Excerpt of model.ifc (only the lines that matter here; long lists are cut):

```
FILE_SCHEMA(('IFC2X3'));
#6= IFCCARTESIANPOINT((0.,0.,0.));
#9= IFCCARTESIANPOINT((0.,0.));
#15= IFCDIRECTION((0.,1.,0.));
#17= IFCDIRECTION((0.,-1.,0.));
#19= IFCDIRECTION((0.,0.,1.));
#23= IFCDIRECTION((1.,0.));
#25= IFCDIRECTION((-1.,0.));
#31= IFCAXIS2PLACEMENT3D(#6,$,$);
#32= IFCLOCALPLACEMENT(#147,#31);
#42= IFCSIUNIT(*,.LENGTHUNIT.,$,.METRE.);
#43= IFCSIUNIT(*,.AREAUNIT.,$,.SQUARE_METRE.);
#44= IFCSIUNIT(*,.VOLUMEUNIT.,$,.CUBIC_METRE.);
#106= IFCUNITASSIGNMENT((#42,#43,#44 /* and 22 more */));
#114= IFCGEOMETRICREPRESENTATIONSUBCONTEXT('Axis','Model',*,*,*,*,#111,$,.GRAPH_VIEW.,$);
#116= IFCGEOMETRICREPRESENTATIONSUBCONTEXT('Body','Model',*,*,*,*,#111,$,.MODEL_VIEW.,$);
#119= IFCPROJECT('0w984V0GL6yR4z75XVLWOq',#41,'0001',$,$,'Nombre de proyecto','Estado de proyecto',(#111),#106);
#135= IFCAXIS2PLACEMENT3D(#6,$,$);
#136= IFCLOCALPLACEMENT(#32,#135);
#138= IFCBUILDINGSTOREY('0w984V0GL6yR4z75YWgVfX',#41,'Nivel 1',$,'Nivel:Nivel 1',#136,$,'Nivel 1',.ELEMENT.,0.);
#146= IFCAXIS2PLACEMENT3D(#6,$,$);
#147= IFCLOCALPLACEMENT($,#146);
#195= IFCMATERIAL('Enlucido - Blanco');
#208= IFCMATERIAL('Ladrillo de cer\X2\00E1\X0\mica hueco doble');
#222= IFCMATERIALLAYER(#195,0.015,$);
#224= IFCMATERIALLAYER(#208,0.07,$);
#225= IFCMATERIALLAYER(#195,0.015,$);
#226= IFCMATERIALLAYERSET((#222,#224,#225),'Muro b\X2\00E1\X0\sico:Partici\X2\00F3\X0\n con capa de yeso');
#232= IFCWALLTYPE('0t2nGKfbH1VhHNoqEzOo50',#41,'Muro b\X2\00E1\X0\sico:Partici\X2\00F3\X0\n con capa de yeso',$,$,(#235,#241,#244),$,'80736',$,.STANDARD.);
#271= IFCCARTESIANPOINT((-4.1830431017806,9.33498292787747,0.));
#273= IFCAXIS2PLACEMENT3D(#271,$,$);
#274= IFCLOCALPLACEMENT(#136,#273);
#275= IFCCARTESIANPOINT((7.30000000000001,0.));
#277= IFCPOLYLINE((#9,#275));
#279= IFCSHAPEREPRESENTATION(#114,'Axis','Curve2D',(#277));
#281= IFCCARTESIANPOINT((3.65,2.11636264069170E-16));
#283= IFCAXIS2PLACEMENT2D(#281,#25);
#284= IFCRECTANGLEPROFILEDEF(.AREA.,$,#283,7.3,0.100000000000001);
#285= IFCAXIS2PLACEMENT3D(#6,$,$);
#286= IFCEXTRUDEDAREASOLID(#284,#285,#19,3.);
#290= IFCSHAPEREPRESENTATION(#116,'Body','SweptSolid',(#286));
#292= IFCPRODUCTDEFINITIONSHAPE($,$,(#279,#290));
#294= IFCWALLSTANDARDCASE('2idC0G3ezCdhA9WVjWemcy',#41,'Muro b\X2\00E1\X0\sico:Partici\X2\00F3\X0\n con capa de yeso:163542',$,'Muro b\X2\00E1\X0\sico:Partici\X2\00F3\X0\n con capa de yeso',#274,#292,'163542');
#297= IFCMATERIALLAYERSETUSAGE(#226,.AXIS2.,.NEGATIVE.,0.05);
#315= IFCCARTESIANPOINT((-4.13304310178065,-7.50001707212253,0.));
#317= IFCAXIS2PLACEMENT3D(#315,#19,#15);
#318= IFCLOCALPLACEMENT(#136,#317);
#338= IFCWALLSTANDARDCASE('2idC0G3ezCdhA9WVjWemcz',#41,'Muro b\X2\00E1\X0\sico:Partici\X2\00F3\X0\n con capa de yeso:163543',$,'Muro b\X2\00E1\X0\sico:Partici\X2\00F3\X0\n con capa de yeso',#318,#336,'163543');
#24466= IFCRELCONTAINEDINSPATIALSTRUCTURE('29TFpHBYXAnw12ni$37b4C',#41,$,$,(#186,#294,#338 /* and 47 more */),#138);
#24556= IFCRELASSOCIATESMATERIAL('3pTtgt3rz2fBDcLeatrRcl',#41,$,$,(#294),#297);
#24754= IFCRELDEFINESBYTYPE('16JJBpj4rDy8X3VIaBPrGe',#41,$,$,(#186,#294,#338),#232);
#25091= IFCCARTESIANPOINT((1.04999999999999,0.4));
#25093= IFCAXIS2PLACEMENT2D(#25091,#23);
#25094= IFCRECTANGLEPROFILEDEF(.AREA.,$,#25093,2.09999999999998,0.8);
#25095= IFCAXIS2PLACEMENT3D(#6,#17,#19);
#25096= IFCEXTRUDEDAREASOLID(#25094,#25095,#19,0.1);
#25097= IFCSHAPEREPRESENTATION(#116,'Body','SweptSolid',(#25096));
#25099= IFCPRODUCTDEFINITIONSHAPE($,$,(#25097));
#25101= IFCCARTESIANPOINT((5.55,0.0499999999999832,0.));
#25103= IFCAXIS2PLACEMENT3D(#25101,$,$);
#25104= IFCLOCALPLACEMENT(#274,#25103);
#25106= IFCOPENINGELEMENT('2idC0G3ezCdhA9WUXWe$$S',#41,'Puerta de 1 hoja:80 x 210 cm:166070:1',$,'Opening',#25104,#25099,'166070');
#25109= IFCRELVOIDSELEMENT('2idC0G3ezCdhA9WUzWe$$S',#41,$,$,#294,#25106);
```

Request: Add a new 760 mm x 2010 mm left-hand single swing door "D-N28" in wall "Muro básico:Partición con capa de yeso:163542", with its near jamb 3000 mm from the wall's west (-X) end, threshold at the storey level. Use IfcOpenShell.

```python
import numpy as np
import ifcopenshell
import ifcopenshell.api.feature
import ifcopenshell.api.geometry
import ifcopenshell.api.root
import ifcopenshell.api.spatial
import ifcopenshell.api.type
import ifcopenshell.geom
import ifcopenshell.util.element
import ifcopenshell.util.placement
import ifcopenshell.util.representation
import ifcopenshell.util.shape
import ifcopenshell.util.unit

model = ifcopenshell.open("model.ifc")
unit_scale = ifcopenshell.util.unit.calculate_unit_scale(model)
settings = ifcopenshell.geom.settings()


def volume(element):
    """Net volume in cubic metres, openings subtracted."""
    shape = ifcopenshell.geom.create_shape(settings, element)
    return ifcopenshell.util.shape.get_volume(shape.geometry)


wall = model.by_guid("2idC0G3ezCdhA9WVjWemcy")
storey = ifcopenshell.util.element.get_container(wall, ifc_class="IfcBuildingStorey")
context = ifcopenshell.util.representation.get_context(model, "Model", "Body", "MODEL_VIEW")
before = volume(wall)

width, height, from_end, sill = 0.76, 2.01, 3, 0.0  # metres

# The wall runs along its own X axis, and the end named is its -X end.
wall_shape = ifcopenshell.geom.create_shape(settings, wall)
x, y, z = ifcopenshell.util.shape.get_vertices(wall_shape.geometry).T
start = x.min() + from_end
face, thickness = float(y.min()), float(y.max() - y.min())
wall_matrix = ifcopenshell.util.placement.get_local_placement(wall.ObjectPlacement)
level = ifcopenshell.util.placement.get_local_placement(storey.ObjectPlacement)[2, 3]


def in_wall(x, y):
    """Placement at x, y metres in the wall's axes, at sill height."""
    matrix = wall_matrix.copy()
    matrix[:, 3] = wall_matrix @ np.array([x / unit_scale, y / unit_scale, 0.0, 1.0])
    matrix[2, 3] = level + sill / unit_scale
    return matrix


# Opening: a box that overshoots both wall faces by 50 mm.
opening = ifcopenshell.api.root.create_entity(model, ifc_class="IfcOpeningElement")
box = ifcopenshell.api.geometry.add_wall_representation(
    model, context=context, length=width, height=height, thickness=thickness + 0.1
)
ifcopenshell.api.geometry.assign_representation(model, product=opening, representation=box)
ifcopenshell.api.geometry.edit_object_placement(model, product=opening, matrix=in_wall(start, face - 0.05), is_si=False)
ifcopenshell.api.feature.add_feature(model, feature=opening, element=wall)

door = ifcopenshell.api.root.create_entity(model, ifc_class="IfcDoor", name="D-N28")
door.OverallWidth, door.OverallHeight = width / unit_scale, height / unit_scale
body = ifcopenshell.api.geometry.add_door_representation(
    model,
    context=context,
    overall_width=door.OverallWidth,
    overall_height=door.OverallHeight,
    operation_type="SINGLE_SWING_LEFT",
    lining_properties={"LiningDepth": thickness / unit_scale, "ThresholdDepth": thickness / unit_scale},
)
ifcopenshell.api.geometry.assign_representation(model, product=door, representation=body)
ifcopenshell.api.spatial.assign_container(model, products=[door], relating_structure=storey)
fills = ifcopenshell.api.feature.add_filling(model, opening=opening, element=door)
fills.OwnerHistory = door.OwnerHistory  # required in IFC2X3

# IFC2X3 keeps the operation on the door style.
style = ifcopenshell.api.root.create_entity(model, ifc_class="IfcDoorStyle", name="D-N28")
style.OperationType, style.ConstructionType = "SINGLE_SWING_LEFT", "NOTDEFINED"
style.ParameterTakesPrecedence = style.Sizeable = False
ifcopenshell.api.type.assign_type(model, related_objects=[door], relating_type=style)

# The lining spans the wall, so the door starts at the wall face.
ifcopenshell.api.geometry.edit_object_placement(model, product=door, matrix=in_wall(start, face), is_si=False)

after = volume(wall)

print(f"wall volume {before:.3f} -> {after:.3f} m3")

model.write("model_edited.ifc")
```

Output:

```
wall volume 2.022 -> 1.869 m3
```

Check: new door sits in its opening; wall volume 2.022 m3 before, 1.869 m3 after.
